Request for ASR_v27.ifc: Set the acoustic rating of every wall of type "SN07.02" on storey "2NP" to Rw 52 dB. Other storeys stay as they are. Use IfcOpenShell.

First a look at what the model holds.

```python
import ifcopenshell
import ifcopenshell.util.element

model = ifcopenshell.open("ASR_v27.ifc")
print(model.schema)
storey = next(s for s in model.by_type("IfcBuildingStorey") if s.Name == "2NP")
walls = [e for e in ifcopenshell.util.element.get_decomposition(storey) if e.is_a("IfcWall")]
seen = {}
for e in walls:
    element_type = ifcopenshell.util.element.get_type(e)
    key = (element_type.Name if element_type != e and element_type else None, ifcopenshell.util.element.get_pset(e, "Pset_WallCommon", "AcousticRating"))
    seen[key] = seen.get(key, 0) + 1
for (name, value), count in sorted(seen.items(), key=str):
    print(count, "x", name, "|", value)
```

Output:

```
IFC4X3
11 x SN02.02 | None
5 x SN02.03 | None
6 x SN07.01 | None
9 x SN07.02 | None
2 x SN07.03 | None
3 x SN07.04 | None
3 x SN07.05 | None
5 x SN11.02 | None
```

```python
import ifcopenshell
import ifcopenshell.api.pset
import ifcopenshell.util.element

model = ifcopenshell.open("ASR_v27.ifc")

storey = next(s for s in model.by_type("IfcBuildingStorey") if s.Name == "2NP")
walls = [e for e in ifcopenshell.util.element.get_decomposition(storey) if e.is_a("IfcWall")]

count = 0
for e in walls:
    element_type = ifcopenshell.util.element.get_type(e)
    if element_type in (None, e) or element_type.Name != "SN07.02":
        continue
    # add_pset returns the element's existing set when there is one.
    pset = ifcopenshell.api.pset.add_pset(model, product=e, name="Pset_WallCommon")
    ifcopenshell.api.pset.edit_pset(model, pset=pset, properties={"AcousticRating": "Rw 52 dB"})
    count += 1

print(count, "walls updated")

model.write("ASR_v27_edited.ifc")
```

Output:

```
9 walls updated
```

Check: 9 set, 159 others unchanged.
